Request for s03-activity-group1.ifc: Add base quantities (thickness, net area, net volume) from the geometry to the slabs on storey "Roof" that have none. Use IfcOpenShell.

First a look at what the model holds.

```python
import ifcopenshell
import ifcopenshell.util.element
import ifcopenshell.util.unit

model = ifcopenshell.open("s03-activity-group1.ifc")
print(model.schema)
for unit_type in ("LENGTHUNIT", "AREAUNIT", "VOLUMEUNIT"):
    print(unit_type, ifcopenshell.util.unit.calculate_unit_scale(model, unit_type))
storey = next(s for s in model.by_type("IfcBuildingStorey") if s.Name == "Roof")
slabs = [e for e in ifcopenshell.util.element.get_decomposition(storey) if e.is_a("IfcSlab")]
for e in sorted(slabs, key=lambda e: e.id()):
    print(e.id(), e.is_a(), e.Name, list(ifcopenshell.util.element.get_psets(e, qtos_only=True)), sep=" | ")
```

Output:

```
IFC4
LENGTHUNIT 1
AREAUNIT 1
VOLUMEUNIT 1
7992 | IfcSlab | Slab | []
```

```python
import ifcopenshell
import ifcopenshell.api.pset
import ifcopenshell.geom
import ifcopenshell.util.element
import ifcopenshell.util.shape
import ifcopenshell.util.unit

model = ifcopenshell.open("s03-activity-group1.ifc")
unit_scale = ifcopenshell.util.unit.calculate_unit_scale(model)
area_scale = ifcopenshell.util.unit.calculate_unit_scale(model, "AREAUNIT")
volume_scale = ifcopenshell.util.unit.calculate_unit_scale(model, "VOLUMEUNIT")
settings = ifcopenshell.geom.settings()

storey = next(s for s in model.by_type("IfcBuildingStorey") if s.Name == "Roof")
slabs = [e for e in ifcopenshell.util.element.get_decomposition(storey) if e.is_a("IfcSlab")]

for e in sorted(slabs, key=lambda e: e.id()):
    if ifcopenshell.util.element.get_psets(e, qtos_only=True, should_inherit=False):
        continue
    # Geometry comes back in metres, in the element's own axes.
    shape = ifcopenshell.geom.create_shape(settings, e)
    values = {
        "Width": ifcopenshell.util.shape.get_z(shape.geometry) / unit_scale,
        "NetArea": ifcopenshell.util.shape.get_footprint_area(shape.geometry) / area_scale,
        "NetVolume": ifcopenshell.util.shape.get_volume(shape.geometry) / volume_scale,
    }
    qto = ifcopenshell.api.pset.add_qto(model, product=e, name="Qto_SlabBaseQuantities")
    ifcopenshell.api.pset.edit_qto(model, qto=qto, properties=values)
    print(e.id(), {k: round(v, 3) for k, v in values.items()})

model.write("s03-activity-group1_updated.ifc")
```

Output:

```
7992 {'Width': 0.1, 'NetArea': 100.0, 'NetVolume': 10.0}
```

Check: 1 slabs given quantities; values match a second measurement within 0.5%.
